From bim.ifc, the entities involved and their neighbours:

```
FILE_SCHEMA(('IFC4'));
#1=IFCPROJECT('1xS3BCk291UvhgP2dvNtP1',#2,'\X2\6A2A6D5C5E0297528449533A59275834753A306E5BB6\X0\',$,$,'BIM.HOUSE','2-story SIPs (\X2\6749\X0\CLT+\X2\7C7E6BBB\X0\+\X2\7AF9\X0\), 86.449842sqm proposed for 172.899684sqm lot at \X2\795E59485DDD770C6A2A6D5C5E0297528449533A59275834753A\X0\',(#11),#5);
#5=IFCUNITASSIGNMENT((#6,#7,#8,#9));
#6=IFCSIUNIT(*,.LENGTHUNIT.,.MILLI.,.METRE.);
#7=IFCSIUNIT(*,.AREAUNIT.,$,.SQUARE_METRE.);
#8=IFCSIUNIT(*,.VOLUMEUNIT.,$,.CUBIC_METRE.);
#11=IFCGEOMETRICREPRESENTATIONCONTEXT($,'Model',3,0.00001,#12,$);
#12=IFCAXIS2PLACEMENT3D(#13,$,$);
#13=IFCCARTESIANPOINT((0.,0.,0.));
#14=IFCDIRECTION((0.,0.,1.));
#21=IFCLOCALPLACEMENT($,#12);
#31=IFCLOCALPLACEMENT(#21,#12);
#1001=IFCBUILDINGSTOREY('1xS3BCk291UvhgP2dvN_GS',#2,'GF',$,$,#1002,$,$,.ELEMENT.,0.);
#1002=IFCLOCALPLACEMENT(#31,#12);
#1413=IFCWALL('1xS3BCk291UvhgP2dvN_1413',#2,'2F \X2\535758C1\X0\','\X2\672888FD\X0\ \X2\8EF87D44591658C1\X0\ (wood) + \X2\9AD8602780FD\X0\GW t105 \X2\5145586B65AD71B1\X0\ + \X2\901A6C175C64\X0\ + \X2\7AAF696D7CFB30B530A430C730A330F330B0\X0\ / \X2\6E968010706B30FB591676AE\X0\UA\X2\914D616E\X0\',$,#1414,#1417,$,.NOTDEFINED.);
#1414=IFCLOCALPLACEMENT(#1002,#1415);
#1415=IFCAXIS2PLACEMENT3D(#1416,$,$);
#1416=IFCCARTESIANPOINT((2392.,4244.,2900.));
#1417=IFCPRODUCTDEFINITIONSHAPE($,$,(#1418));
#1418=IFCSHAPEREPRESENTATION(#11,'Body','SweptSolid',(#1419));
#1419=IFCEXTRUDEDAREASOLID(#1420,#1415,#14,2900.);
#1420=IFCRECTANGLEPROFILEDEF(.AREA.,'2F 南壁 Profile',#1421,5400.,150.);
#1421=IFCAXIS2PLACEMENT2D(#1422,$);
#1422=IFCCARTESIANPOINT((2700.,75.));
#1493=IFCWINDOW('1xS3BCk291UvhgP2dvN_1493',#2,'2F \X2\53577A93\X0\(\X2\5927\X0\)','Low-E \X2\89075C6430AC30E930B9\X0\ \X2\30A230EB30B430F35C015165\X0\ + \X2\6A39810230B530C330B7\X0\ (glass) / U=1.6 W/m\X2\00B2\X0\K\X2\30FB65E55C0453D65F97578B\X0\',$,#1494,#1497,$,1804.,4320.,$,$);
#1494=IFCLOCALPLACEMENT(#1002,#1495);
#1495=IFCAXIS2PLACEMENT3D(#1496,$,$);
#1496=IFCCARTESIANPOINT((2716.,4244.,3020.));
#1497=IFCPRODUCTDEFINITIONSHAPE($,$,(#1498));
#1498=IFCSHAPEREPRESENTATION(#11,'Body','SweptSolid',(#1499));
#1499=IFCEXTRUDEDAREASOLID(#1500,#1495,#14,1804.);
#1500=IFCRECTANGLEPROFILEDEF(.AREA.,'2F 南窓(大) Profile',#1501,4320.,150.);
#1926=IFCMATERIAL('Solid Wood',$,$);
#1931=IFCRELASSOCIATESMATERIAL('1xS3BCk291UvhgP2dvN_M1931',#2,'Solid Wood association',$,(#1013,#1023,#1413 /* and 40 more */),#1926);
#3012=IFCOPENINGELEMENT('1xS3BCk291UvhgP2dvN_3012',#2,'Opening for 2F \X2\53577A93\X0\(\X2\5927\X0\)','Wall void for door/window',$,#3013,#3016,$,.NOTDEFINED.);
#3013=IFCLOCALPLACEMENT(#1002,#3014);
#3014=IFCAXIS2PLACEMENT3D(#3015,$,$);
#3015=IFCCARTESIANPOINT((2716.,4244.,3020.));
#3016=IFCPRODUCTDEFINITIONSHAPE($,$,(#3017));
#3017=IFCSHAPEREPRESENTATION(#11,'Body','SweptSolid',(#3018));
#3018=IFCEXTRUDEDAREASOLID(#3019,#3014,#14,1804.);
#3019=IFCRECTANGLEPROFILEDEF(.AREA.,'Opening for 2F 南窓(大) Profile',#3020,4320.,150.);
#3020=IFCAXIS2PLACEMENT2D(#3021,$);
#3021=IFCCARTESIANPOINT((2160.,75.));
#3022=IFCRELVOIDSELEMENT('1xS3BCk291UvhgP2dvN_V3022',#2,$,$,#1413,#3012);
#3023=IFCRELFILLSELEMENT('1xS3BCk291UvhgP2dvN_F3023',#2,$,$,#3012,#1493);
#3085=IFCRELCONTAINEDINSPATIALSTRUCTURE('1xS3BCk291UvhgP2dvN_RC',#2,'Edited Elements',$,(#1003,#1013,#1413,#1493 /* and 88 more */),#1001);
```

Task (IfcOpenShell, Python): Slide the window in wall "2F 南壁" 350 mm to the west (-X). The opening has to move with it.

```python
import ifcopenshell
import ifcopenshell.api.geometry
import ifcopenshell.util.placement
import ifcopenshell.util.unit

model = ifcopenshell.open("bim.ifc")
unit_scale = ifcopenshell.util.unit.calculate_unit_scale(model)

window = model.by_guid("1xS3BCk291UvhgP2dvN_1493")
opening = window.FillsVoids[0].RelatingOpeningElement
wall = opening.VoidsElements[0].RelatingBuildingElement

wall_matrix = ifcopenshell.util.placement.get_local_placement(wall.ObjectPlacement)
shift = wall_matrix[:3, 0] * -0.35 / unit_scale
before = ifcopenshell.util.placement.get_local_placement(window.ObjectPlacement)[:3, 3].copy()

# The window is not placed relative to its opening, so move both.
for product in (opening, window):
    matrix = ifcopenshell.util.placement.get_local_placement(product.ObjectPlacement)
    matrix[:3, 3] += shift
    ifcopenshell.api.geometry.edit_object_placement(model, product=product, matrix=matrix, is_si=False)

after = ifcopenshell.util.placement.get_local_placement(window.ObjectPlacement)[:3, 3]
print("window moved by", (after - before).round(3) + 0.0)

model.write("bim_edited.ifc")
```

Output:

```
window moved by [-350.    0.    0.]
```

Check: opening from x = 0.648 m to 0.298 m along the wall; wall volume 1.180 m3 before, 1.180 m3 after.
